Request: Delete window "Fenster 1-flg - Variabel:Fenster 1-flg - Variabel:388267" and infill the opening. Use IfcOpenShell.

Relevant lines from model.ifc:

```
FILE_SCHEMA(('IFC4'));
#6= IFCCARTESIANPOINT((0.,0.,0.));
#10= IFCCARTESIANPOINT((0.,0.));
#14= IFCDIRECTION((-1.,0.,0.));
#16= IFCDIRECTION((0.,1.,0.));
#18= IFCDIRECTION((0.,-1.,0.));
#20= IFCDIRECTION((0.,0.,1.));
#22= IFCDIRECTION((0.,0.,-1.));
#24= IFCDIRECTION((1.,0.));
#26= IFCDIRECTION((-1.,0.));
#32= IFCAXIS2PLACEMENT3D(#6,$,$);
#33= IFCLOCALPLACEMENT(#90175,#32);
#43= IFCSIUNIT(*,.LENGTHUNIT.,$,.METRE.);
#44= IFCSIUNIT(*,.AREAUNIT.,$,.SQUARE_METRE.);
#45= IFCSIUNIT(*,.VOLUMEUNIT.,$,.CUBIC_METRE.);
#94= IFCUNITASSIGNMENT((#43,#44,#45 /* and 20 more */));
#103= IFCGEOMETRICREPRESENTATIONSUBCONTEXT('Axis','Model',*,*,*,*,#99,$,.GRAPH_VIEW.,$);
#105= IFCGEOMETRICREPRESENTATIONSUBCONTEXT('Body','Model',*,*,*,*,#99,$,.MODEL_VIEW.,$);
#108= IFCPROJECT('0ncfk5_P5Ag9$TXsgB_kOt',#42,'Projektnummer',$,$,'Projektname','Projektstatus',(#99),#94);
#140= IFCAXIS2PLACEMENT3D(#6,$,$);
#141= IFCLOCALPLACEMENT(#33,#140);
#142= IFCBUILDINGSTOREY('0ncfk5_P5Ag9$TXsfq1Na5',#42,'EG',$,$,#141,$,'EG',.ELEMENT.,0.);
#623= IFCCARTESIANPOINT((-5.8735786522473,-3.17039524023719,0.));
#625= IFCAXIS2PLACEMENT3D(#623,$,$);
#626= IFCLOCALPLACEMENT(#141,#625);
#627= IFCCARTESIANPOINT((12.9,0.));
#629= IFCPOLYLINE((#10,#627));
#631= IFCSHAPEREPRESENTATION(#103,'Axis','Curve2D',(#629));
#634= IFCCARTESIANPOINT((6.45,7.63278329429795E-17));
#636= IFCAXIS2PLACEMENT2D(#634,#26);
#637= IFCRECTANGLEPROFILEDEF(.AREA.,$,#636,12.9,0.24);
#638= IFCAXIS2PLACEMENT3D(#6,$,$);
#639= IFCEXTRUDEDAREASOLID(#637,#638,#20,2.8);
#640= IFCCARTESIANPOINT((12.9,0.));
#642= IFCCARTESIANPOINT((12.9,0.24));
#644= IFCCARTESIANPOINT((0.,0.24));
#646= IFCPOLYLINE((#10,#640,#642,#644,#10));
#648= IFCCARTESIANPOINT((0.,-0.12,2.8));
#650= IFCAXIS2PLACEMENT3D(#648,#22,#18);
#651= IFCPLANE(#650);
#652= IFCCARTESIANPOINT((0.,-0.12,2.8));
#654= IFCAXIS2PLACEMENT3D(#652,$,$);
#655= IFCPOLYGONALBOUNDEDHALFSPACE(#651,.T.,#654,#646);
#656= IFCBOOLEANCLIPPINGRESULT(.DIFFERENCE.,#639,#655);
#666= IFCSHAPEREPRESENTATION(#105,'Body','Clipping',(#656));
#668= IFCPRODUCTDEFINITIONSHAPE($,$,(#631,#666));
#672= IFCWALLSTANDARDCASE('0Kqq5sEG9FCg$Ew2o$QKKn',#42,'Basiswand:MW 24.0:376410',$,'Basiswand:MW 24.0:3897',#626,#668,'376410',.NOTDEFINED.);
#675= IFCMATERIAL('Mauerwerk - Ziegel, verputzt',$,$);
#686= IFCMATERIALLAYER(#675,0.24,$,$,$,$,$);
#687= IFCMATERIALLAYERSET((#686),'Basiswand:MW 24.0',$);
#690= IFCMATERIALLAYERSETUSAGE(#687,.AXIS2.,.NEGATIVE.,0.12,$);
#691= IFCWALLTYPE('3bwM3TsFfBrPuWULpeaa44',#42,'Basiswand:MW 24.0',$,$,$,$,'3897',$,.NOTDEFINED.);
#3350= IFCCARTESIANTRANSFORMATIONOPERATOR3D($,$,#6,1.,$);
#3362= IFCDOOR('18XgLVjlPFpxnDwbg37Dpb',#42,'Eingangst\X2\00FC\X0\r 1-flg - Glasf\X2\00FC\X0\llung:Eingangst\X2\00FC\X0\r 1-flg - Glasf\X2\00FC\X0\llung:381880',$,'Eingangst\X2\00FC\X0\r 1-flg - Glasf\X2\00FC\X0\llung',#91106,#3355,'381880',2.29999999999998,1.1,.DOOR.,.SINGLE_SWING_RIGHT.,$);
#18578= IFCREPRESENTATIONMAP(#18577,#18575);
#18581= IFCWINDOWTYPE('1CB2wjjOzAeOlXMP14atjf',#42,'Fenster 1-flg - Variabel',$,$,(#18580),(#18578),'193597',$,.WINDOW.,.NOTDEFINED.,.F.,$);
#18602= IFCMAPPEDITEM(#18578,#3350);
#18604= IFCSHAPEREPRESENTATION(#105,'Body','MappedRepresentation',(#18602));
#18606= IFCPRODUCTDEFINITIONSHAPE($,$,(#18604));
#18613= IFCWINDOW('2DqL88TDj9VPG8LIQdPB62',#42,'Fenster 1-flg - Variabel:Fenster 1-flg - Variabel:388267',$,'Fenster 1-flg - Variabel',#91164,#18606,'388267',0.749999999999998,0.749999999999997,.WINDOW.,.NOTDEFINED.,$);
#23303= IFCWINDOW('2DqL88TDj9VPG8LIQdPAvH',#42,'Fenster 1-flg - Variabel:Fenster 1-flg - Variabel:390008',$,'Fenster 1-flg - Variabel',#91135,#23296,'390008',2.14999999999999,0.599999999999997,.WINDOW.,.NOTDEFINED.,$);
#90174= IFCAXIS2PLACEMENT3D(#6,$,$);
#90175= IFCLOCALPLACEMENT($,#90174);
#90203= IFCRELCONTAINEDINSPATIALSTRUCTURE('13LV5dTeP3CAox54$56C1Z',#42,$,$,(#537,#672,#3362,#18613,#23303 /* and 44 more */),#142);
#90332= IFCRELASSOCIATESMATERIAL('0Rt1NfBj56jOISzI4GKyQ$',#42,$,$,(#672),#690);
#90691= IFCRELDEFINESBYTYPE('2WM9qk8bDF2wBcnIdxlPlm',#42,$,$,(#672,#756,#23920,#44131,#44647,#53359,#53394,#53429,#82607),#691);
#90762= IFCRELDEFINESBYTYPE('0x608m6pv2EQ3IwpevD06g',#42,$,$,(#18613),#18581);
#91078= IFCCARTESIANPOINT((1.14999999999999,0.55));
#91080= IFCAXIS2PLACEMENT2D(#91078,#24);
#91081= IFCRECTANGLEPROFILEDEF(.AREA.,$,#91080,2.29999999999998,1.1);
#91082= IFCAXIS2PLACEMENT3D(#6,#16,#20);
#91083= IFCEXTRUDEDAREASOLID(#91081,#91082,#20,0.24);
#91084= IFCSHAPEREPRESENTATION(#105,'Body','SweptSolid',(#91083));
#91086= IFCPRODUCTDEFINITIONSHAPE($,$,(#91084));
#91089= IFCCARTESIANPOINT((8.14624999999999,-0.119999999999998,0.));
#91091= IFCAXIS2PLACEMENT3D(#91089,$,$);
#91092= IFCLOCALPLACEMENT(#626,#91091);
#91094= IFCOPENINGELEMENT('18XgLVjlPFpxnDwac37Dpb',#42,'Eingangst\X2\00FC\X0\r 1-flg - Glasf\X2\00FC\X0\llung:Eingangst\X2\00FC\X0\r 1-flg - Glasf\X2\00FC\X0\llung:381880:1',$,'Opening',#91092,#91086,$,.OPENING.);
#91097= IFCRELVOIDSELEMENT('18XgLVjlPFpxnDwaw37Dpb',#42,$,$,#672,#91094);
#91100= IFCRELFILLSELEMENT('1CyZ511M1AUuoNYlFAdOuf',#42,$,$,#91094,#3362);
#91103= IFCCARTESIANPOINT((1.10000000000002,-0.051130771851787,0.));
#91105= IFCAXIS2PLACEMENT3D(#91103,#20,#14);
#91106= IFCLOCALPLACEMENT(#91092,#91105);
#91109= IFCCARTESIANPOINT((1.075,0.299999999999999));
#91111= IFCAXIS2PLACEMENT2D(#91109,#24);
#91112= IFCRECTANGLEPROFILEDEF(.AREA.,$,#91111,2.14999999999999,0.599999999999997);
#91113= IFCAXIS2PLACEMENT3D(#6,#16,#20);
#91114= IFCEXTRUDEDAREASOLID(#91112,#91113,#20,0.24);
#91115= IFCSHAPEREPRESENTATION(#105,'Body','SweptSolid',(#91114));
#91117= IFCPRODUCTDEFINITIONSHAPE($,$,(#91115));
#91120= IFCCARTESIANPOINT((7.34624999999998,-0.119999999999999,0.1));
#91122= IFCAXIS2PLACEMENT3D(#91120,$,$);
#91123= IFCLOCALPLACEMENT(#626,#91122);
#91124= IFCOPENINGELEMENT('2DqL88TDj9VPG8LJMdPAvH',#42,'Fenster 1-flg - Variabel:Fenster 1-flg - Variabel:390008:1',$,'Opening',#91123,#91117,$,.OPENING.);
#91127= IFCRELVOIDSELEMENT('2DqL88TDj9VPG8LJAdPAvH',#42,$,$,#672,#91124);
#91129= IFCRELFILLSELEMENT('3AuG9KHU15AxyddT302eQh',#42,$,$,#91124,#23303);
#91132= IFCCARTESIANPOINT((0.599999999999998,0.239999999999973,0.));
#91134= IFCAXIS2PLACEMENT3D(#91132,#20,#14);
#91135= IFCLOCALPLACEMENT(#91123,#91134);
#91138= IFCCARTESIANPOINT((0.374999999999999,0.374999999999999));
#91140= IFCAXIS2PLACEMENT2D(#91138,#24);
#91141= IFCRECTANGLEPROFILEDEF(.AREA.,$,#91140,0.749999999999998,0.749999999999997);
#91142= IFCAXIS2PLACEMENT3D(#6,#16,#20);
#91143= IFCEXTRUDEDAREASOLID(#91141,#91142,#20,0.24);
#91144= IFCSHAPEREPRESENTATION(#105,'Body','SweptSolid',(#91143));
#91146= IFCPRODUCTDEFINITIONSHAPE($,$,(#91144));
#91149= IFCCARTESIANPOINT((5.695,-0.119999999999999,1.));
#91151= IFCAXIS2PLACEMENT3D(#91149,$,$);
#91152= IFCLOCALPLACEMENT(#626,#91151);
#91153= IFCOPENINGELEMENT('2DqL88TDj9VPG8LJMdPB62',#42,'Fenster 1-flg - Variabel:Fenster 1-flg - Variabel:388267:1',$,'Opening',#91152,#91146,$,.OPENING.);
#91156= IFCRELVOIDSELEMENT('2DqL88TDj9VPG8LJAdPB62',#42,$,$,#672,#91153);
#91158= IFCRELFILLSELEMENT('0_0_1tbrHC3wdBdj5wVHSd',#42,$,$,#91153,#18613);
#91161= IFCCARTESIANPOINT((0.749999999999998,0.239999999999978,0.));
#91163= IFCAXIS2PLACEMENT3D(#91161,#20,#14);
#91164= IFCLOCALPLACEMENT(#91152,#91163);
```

```python
import ifcopenshell
import ifcopenshell.api.feature
import ifcopenshell.api.root
import ifcopenshell.geom
import ifcopenshell.util.shape

model = ifcopenshell.open("model.ifc")
settings = ifcopenshell.geom.settings()


def volume(element):
    """Net volume in cubic metres, openings subtracted."""
    shape = ifcopenshell.geom.create_shape(settings, element)
    return ifcopenshell.util.shape.get_volume(shape.geometry)


window = model.by_guid("2DqL88TDj9VPG8LIQdPB62")
opening = window.FillsVoids[0].RelatingOpeningElement
wall = opening.VoidsElements[0].RelatingBuildingElement
before = volume(wall)

ifcopenshell.api.root.remove_product(model, product=window)
ifcopenshell.api.feature.remove_feature(model, feature=opening)

after = volume(wall)

print(f"wall volume {before:.3f} -> {after:.3f} m3")

model.write("model_updated.ifc")
```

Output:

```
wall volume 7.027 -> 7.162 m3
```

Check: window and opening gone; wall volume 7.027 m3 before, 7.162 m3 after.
